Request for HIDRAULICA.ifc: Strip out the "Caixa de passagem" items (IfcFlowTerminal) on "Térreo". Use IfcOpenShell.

First a look at what the model holds.

```python
import ifcopenshell
import ifcopenshell.util.element

model = ifcopenshell.open("HIDRAULICA.ifc")
print(model.schema)
storey = next(s for s in model.by_type("IfcBuildingStorey") if s.Name == "Térreo")
terminals = [e for e in ifcopenshell.util.element.get_decomposition(storey) if e.is_a("IfcFlowTerminal")]
seen = {}
for e in terminals:
    element_type = ifcopenshell.util.element.get_type(e)
    name = element_type.Name if element_type not in (None, e) else None
    seen[name] = seen.get(name, 0) + 1
for name, count in sorted(seen.items(), key=str):
    print(count, "x", name)
```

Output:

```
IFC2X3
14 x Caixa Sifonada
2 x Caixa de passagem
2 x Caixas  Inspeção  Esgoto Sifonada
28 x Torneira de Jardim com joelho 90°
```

```python
import ifcopenshell
import ifcopenshell.api.root
import ifcopenshell.util.element

model = ifcopenshell.open("HIDRAULICA.ifc")

storey = next(s for s in model.by_type("IfcBuildingStorey") if s.Name == "Térreo")
terminals = [e for e in ifcopenshell.util.element.get_decomposition(storey) if e.is_a("IfcFlowTerminal")]
targets = [e for e in terminals if (t := ifcopenshell.util.element.get_type(e)) not in (None, e) and t.Name == "Caixa de passagem"]

for e in targets:
    ifcopenshell.api.root.remove_product(model, product=e)
print(len(targets), "removed")

model.write("HIDRAULICA_rev.ifc")
```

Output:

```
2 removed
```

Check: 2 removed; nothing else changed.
